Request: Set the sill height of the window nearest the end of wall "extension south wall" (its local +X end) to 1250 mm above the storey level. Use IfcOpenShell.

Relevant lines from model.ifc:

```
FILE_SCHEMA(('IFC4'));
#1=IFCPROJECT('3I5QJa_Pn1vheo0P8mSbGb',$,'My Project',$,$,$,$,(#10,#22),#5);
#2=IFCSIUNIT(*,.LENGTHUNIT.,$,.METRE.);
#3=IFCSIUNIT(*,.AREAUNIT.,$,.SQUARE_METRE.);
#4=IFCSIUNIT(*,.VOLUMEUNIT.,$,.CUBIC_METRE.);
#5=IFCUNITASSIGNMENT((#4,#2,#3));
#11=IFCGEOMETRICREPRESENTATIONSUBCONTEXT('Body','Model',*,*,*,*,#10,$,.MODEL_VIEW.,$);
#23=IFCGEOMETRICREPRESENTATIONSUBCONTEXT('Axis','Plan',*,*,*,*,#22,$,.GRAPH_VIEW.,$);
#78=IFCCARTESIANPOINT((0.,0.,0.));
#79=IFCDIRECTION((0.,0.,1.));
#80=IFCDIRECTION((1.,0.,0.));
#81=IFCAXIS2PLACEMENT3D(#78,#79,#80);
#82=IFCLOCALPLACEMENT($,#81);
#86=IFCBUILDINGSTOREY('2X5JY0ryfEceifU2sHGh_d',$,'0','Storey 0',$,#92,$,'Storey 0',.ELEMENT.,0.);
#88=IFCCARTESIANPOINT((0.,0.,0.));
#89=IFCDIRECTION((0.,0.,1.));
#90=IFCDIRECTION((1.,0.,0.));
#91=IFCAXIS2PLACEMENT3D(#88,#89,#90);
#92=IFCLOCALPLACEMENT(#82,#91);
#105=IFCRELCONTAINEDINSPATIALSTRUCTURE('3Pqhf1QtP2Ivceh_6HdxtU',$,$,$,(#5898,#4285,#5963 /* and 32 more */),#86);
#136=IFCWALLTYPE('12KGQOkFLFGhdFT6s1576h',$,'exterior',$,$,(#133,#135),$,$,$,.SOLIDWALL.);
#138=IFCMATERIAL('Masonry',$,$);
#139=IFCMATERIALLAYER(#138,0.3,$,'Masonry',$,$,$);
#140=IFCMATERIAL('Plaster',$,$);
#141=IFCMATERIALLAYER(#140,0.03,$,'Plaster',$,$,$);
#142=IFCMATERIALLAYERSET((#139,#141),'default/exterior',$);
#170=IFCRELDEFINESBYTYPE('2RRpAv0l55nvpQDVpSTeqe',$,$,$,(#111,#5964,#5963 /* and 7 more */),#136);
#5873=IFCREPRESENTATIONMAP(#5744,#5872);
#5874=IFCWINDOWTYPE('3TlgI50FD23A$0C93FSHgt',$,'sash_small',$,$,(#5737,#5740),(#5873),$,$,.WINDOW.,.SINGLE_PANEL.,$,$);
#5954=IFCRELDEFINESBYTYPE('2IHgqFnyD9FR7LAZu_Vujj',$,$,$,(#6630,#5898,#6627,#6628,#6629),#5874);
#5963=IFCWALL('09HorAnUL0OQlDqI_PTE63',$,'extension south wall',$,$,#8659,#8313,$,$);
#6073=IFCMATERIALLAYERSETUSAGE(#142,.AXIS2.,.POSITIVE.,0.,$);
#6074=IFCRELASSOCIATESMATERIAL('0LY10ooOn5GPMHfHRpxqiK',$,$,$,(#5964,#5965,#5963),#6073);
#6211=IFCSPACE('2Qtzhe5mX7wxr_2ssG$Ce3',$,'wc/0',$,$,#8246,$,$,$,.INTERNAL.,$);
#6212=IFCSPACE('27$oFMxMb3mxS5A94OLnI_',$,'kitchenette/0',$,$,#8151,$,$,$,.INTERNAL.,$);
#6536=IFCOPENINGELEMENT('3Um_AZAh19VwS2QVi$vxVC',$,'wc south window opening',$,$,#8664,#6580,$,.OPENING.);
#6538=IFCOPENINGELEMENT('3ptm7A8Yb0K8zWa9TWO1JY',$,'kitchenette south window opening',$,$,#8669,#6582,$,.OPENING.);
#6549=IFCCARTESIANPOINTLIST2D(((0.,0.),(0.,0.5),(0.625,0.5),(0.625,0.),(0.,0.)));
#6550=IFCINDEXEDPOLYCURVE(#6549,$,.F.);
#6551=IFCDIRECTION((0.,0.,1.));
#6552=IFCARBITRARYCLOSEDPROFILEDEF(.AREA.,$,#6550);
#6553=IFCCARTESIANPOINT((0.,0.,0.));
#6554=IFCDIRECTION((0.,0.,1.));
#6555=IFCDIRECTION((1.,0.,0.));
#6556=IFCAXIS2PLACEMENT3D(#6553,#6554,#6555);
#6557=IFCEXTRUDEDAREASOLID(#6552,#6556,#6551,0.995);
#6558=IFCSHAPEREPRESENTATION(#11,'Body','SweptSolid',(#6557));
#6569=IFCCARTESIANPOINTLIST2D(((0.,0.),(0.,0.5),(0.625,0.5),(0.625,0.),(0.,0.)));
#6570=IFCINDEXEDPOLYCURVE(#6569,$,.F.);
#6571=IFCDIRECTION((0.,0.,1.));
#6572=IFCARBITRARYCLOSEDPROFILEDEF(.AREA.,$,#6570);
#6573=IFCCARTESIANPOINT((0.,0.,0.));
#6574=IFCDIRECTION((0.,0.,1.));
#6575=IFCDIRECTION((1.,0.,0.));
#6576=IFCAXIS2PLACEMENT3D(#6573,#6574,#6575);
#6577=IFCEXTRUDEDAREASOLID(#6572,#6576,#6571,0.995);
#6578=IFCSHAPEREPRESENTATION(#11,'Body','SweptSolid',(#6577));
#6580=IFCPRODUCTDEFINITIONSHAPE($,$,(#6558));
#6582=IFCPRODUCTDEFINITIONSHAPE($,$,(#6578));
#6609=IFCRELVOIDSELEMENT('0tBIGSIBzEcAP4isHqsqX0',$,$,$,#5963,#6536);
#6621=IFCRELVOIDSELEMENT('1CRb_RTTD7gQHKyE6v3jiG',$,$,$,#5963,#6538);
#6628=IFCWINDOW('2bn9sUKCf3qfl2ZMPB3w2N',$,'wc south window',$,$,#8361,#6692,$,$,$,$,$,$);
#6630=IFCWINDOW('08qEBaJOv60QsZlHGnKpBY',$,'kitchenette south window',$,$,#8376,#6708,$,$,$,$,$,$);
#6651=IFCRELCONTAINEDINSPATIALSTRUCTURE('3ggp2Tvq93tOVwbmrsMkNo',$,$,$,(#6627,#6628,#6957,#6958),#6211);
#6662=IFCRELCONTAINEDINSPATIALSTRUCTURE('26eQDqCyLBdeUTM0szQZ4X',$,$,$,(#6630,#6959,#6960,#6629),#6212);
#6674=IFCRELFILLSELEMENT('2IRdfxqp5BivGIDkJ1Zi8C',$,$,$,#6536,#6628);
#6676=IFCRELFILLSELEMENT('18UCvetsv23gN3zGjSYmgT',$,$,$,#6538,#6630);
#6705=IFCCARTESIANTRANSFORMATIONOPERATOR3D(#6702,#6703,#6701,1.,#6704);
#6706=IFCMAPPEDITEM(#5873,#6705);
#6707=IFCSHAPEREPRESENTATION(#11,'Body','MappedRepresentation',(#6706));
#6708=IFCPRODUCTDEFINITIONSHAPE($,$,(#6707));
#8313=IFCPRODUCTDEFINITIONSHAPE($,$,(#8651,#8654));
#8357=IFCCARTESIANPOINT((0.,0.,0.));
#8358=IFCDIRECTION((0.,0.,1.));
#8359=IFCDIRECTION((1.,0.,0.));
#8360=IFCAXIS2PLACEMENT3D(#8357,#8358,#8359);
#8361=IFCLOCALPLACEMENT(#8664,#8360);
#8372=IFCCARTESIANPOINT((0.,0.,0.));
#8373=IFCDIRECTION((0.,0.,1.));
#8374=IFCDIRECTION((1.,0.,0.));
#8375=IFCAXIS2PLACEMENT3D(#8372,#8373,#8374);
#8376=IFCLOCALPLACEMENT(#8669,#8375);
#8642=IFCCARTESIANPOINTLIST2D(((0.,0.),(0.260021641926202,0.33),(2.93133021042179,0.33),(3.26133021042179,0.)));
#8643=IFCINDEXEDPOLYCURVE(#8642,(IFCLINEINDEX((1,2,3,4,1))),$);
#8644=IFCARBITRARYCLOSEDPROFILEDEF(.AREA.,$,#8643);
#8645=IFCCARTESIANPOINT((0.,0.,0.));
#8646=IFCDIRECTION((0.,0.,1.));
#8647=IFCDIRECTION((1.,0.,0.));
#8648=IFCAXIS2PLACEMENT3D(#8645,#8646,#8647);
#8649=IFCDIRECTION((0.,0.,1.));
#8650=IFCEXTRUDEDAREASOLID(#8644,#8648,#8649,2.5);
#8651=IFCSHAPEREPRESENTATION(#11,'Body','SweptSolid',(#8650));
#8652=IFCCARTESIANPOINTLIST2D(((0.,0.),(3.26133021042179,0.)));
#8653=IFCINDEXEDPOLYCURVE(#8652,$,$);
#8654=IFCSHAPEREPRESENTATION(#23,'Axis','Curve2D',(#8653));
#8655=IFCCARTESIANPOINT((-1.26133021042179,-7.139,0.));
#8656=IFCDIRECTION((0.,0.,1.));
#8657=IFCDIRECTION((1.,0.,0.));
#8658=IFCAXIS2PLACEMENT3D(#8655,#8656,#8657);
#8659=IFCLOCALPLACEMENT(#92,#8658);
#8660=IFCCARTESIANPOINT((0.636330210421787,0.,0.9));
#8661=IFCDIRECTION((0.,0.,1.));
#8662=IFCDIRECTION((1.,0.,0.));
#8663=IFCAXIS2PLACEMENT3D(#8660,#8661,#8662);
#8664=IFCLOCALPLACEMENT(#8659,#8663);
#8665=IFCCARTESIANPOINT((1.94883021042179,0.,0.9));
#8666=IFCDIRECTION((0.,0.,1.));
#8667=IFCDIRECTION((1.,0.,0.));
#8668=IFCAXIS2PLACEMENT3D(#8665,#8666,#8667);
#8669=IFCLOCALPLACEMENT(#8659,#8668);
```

```python
import numpy as np
import ifcopenshell
import ifcopenshell.api.geometry
import ifcopenshell.geom
import ifcopenshell.util.element
import ifcopenshell.util.placement
import ifcopenshell.util.shape
import ifcopenshell.util.unit

model = ifcopenshell.open("model.ifc")
unit_scale = ifcopenshell.util.unit.calculate_unit_scale(model)

window = model.by_guid("08qEBaJOv60QsZlHGnKpBY")
opening = window.FillsVoids[0].RelatingOpeningElement
storey = ifcopenshell.util.element.get_container(window, ifc_class="IfcBuildingStorey")
level = ifcopenshell.util.placement.get_local_placement(storey.ObjectPlacement)[2, 3]

# The opening's origin need not be at the sill, so measure its lowest point.
shape = ifcopenshell.geom.create_shape(ifcopenshell.geom.settings(), opening)
bottom = ifcopenshell.util.shape.get_shape_bottom_elevation(shape, shape.geometry) / unit_scale
dz = level + 1.25 / unit_scale - bottom

shift = np.array([0.0, 0.0, dz])
# The window is placed relative to its opening, so it follows when the opening moves.
matrix = ifcopenshell.util.placement.get_local_placement(opening.ObjectPlacement)
matrix[:3, 3] += shift
ifcopenshell.api.geometry.edit_object_placement(
    model, product=opening, matrix=matrix, is_si=False, should_transform_children=True
)

print(f"moved by {dz * unit_scale:+.3f} m")

model.write("model_updated.ifc")
```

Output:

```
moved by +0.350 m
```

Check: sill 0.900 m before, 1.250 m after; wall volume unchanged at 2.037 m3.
